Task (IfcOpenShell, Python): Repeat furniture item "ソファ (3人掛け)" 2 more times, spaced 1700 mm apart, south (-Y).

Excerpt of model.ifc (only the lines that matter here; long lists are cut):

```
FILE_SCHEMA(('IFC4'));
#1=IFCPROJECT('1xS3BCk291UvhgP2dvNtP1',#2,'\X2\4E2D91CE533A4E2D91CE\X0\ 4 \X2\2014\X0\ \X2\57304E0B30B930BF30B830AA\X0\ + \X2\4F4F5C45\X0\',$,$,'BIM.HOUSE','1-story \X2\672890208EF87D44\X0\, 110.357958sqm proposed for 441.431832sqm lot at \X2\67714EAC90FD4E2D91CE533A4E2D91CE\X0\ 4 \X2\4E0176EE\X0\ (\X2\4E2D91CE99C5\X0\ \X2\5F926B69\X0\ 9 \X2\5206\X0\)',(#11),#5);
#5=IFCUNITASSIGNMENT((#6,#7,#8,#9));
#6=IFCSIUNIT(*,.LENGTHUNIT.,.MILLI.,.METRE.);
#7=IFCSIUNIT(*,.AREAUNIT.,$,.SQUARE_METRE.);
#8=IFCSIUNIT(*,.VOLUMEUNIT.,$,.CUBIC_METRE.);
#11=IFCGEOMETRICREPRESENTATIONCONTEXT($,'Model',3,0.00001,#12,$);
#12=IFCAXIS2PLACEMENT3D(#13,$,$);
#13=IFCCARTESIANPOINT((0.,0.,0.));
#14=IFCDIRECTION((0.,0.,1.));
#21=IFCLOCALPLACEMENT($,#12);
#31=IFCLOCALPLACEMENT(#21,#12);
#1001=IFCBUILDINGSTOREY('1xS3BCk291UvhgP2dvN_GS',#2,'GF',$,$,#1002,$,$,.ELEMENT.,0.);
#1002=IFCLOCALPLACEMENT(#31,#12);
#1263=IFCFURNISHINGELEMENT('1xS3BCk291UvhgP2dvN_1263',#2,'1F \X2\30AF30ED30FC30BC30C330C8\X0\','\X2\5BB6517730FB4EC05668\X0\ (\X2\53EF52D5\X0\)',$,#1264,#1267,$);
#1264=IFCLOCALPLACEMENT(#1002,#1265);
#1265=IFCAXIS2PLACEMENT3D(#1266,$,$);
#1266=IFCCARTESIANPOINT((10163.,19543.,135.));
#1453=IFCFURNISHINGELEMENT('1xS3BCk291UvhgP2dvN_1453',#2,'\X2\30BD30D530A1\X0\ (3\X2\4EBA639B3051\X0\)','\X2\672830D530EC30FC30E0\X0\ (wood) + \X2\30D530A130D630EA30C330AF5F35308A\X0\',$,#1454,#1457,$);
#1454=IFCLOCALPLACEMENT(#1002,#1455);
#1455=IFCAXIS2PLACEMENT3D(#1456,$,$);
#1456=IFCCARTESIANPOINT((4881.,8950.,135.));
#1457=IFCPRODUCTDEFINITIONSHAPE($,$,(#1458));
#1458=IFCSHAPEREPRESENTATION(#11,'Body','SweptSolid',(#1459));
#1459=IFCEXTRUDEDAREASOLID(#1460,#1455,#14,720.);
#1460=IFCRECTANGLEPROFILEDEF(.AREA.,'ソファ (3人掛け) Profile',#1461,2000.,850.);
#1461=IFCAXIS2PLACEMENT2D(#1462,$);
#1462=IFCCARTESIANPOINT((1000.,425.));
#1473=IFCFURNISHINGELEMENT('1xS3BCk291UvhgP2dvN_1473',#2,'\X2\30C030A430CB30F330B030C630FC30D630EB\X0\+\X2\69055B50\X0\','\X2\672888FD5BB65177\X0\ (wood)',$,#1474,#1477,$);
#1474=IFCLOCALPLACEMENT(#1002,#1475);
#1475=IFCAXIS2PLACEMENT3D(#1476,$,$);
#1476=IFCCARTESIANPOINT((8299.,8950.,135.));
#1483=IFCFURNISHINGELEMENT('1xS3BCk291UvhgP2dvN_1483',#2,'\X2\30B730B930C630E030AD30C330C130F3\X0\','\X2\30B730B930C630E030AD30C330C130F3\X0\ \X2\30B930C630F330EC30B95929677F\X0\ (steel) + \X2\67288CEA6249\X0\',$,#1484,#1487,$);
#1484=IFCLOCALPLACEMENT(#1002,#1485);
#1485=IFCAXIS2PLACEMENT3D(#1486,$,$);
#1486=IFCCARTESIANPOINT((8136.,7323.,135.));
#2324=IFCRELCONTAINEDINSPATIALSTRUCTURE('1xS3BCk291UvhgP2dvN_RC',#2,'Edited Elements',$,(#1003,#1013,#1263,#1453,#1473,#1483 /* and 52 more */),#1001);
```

```python
import numpy as np
import ifcopenshell
import ifcopenshell.api.geometry
import ifcopenshell.api.root
import ifcopenshell.util.element
import ifcopenshell.util.placement

model = ifcopenshell.open("model.ifc")


def reuse_history(source, copy):
    """copy_class also copies each property set's owner history, people and application; keep the originals."""
    for rel in copy.IsDefinedBy:
        if rel.is_a("IfcRelDefinesByProperties") and (history := rel.RelatingPropertyDefinition.OwnerHistory):
            rel.RelatingPropertyDefinition.OwnerHistory = source.OwnerHistory
            ifcopenshell.util.element.remove_deep2(model, history)


source = model.by_guid("1xS3BCk291UvhgP2dvN_1453")
base = ifcopenshell.util.placement.get_local_placement(source.ObjectPlacement)
step = np.array([0.0, -1.0, 0.0]) * 1700.0

for i in range(1, 3):
    copy = ifcopenshell.api.root.copy_class(model, product=source)
    copy.Representation = ifcopenshell.util.element.copy_deep(
        model, source.Representation, exclude=["IfcGeometricRepresentationContext", "IfcRepresentationMap"]
    )
    reuse_history(source, copy)
    matrix = base.copy()
    matrix[:3, 3] += i * step
    print("added at", matrix[:3, 3].round(3) + 0.0)
    ifcopenshell.api.geometry.edit_object_placement(model, product=copy, matrix=matrix, is_si=False)

model.write("model_updated.ifc")
```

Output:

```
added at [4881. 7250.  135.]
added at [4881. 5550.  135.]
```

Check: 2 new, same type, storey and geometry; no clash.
